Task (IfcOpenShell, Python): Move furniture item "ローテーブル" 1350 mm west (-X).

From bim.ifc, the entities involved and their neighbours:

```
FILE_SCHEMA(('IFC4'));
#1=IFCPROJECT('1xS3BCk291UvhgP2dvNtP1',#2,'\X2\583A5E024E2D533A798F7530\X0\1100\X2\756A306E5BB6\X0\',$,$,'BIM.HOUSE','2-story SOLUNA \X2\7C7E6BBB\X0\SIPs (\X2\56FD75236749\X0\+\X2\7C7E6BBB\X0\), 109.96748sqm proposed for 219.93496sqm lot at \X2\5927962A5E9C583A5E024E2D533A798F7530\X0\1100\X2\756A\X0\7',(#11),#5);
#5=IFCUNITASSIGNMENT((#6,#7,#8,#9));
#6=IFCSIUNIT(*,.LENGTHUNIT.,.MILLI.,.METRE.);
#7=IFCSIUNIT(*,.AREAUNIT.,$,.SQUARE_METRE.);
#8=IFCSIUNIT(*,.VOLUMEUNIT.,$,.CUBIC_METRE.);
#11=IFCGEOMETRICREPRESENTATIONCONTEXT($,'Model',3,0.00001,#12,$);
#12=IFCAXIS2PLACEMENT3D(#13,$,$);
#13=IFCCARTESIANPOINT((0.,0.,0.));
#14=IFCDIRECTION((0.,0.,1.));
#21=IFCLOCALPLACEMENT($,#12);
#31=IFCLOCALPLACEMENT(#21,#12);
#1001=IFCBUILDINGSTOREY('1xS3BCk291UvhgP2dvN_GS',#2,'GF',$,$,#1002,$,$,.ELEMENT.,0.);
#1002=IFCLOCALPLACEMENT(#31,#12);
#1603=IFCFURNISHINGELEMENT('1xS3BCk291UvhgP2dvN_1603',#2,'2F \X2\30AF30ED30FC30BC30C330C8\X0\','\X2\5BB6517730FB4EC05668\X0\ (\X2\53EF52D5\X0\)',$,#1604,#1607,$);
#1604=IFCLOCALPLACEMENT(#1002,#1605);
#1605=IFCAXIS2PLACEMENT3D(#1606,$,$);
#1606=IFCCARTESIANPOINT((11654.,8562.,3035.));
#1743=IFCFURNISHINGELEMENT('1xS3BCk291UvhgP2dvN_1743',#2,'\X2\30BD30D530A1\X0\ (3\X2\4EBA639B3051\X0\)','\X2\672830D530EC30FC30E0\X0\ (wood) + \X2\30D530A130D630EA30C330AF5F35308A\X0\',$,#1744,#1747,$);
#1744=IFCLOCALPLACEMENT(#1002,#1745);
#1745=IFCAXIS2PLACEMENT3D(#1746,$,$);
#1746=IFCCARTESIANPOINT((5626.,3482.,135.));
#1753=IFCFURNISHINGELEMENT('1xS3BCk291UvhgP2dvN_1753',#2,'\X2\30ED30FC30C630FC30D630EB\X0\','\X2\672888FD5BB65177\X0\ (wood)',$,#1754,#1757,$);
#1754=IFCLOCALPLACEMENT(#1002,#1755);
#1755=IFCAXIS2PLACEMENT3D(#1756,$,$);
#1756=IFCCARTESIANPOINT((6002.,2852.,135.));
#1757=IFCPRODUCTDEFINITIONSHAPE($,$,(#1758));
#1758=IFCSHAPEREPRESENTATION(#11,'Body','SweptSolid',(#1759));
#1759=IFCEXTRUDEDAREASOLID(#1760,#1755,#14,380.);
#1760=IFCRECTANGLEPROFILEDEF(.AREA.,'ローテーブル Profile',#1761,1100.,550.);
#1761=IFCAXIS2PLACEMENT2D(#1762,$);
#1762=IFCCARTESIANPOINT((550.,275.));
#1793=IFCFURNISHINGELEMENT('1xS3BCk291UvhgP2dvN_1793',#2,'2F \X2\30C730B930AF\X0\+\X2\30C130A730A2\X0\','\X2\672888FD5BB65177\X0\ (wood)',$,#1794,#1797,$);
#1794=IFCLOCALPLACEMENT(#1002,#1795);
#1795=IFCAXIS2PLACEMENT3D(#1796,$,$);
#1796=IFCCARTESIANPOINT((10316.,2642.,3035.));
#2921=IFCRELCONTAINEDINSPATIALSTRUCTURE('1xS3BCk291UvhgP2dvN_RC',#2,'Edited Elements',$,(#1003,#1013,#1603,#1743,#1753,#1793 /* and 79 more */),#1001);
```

```python
import ifcopenshell
import ifcopenshell.api.geometry
import ifcopenshell.util.placement

model = ifcopenshell.open("bim.ifc")

item = model.by_id(1753)
matrix = ifcopenshell.util.placement.get_local_placement(item.ObjectPlacement)
matrix[0, 3] -= 1350.0
ifcopenshell.api.geometry.edit_object_placement(model, product=item, matrix=matrix, is_si=False)

print(ifcopenshell.util.placement.get_local_placement(item.ObjectPlacement).round(3) + 0.0)

model.write("bim_rev.ifc")
```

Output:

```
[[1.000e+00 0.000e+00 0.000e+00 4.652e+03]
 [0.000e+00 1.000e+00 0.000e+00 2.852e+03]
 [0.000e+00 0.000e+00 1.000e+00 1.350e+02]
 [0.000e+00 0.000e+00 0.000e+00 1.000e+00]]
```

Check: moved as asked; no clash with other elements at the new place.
